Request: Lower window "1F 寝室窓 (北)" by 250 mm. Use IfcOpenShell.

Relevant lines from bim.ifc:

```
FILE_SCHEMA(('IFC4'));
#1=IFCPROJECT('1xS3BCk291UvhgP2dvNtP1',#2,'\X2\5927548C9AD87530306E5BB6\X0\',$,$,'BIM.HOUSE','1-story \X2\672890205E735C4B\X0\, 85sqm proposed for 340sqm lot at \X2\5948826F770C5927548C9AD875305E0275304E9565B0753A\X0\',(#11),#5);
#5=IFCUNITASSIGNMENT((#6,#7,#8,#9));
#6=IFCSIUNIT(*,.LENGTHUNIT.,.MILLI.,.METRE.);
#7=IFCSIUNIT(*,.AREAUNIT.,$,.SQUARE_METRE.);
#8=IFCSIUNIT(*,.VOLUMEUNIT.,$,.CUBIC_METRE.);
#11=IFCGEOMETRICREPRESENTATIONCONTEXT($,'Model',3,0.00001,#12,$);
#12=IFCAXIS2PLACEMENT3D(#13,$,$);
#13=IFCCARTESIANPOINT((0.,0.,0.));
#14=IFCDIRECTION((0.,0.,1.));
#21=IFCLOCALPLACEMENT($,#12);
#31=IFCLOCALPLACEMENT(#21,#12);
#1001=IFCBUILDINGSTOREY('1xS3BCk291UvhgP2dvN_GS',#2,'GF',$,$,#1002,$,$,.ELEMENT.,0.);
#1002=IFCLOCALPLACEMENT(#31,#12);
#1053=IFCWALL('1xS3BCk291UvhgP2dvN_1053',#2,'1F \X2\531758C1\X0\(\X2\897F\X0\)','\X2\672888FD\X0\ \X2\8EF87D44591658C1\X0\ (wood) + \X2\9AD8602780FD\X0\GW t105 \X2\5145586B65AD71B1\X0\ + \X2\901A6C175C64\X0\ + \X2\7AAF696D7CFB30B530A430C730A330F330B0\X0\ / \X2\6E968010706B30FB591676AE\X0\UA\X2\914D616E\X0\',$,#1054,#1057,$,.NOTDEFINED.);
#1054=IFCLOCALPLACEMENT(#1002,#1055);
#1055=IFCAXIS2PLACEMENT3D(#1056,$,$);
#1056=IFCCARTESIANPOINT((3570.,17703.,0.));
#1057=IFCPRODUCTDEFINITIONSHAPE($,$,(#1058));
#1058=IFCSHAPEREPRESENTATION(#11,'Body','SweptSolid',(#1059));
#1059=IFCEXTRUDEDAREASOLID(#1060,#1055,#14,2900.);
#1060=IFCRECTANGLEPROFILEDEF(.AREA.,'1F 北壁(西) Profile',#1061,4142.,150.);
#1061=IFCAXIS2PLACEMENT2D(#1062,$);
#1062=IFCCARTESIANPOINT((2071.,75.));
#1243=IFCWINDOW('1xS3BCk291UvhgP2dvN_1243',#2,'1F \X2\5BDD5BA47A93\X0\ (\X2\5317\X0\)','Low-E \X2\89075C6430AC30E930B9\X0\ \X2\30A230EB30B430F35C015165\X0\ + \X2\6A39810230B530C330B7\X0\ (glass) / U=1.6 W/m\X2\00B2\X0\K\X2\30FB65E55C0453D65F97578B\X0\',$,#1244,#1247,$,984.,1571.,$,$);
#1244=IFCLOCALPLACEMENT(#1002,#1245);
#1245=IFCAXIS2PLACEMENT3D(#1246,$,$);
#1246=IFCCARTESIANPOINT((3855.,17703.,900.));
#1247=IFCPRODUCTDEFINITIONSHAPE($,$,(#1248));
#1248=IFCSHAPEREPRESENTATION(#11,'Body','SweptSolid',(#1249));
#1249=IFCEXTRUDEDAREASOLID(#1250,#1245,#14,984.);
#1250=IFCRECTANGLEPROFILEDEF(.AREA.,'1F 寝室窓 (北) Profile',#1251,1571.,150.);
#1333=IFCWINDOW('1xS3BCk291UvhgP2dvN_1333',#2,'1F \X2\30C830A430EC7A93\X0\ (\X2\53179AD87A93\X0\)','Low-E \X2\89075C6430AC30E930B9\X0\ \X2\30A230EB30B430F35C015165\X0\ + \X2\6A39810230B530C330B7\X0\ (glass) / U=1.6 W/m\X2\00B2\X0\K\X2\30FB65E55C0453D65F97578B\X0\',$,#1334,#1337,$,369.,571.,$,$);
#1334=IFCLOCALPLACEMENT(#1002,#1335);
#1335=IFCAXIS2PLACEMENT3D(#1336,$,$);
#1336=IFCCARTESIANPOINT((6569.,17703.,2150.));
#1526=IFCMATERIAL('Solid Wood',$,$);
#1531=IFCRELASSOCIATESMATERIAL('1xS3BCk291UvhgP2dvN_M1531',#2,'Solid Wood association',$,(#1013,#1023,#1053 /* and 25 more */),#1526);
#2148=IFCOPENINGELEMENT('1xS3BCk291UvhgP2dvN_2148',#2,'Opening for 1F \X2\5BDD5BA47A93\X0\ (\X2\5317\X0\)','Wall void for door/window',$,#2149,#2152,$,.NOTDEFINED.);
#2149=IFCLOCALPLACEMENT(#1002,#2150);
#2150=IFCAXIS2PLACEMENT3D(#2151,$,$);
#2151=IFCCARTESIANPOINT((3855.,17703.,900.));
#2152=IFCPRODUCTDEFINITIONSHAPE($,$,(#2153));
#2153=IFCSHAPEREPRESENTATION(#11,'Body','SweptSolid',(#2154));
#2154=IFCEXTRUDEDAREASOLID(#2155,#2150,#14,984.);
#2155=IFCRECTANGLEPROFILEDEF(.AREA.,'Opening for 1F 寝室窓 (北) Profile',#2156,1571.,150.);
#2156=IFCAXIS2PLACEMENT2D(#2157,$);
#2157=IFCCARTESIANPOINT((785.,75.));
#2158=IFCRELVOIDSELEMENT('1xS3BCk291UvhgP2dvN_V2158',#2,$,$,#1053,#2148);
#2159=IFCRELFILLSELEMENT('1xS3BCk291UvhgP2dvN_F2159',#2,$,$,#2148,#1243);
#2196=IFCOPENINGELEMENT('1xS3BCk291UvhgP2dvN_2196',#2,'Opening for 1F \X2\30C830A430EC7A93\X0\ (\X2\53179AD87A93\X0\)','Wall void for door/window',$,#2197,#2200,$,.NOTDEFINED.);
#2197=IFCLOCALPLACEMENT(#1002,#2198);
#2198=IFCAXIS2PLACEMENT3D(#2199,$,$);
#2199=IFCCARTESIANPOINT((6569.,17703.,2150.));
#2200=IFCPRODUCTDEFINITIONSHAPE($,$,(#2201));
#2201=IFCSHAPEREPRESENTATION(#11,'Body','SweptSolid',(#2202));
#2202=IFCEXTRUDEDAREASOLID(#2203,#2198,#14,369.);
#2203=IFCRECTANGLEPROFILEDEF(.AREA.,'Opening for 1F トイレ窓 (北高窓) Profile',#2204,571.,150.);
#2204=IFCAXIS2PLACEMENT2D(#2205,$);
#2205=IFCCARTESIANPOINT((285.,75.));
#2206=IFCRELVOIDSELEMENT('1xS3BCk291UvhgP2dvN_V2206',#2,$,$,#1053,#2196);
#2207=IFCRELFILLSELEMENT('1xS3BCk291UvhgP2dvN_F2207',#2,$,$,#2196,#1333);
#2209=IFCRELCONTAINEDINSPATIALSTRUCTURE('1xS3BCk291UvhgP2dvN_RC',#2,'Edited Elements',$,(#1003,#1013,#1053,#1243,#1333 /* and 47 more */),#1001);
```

```python
import numpy as np
import ifcopenshell
import ifcopenshell.api.geometry
import ifcopenshell.util.placement
import ifcopenshell.util.unit

model = ifcopenshell.open("bim.ifc")
unit_scale = ifcopenshell.util.unit.calculate_unit_scale(model)

window = model.by_guid("1xS3BCk291UvhgP2dvN_1243")
opening = window.FillsVoids[0].RelatingOpeningElement
dz = -0.25 / unit_scale

shift = np.array([0.0, 0.0, dz])
# The window is not placed relative to its opening, so move both.
for product in (opening, window):
    matrix = ifcopenshell.util.placement.get_local_placement(product.ObjectPlacement)
    matrix[:3, 3] += shift
    ifcopenshell.api.geometry.edit_object_placement(model, product=product, matrix=matrix, is_si=False)

print(f"moved by {dz * unit_scale:+.3f} m")

model.write("bim_updated.ifc")
```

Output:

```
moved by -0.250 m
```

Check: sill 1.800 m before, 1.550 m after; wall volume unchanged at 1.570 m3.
